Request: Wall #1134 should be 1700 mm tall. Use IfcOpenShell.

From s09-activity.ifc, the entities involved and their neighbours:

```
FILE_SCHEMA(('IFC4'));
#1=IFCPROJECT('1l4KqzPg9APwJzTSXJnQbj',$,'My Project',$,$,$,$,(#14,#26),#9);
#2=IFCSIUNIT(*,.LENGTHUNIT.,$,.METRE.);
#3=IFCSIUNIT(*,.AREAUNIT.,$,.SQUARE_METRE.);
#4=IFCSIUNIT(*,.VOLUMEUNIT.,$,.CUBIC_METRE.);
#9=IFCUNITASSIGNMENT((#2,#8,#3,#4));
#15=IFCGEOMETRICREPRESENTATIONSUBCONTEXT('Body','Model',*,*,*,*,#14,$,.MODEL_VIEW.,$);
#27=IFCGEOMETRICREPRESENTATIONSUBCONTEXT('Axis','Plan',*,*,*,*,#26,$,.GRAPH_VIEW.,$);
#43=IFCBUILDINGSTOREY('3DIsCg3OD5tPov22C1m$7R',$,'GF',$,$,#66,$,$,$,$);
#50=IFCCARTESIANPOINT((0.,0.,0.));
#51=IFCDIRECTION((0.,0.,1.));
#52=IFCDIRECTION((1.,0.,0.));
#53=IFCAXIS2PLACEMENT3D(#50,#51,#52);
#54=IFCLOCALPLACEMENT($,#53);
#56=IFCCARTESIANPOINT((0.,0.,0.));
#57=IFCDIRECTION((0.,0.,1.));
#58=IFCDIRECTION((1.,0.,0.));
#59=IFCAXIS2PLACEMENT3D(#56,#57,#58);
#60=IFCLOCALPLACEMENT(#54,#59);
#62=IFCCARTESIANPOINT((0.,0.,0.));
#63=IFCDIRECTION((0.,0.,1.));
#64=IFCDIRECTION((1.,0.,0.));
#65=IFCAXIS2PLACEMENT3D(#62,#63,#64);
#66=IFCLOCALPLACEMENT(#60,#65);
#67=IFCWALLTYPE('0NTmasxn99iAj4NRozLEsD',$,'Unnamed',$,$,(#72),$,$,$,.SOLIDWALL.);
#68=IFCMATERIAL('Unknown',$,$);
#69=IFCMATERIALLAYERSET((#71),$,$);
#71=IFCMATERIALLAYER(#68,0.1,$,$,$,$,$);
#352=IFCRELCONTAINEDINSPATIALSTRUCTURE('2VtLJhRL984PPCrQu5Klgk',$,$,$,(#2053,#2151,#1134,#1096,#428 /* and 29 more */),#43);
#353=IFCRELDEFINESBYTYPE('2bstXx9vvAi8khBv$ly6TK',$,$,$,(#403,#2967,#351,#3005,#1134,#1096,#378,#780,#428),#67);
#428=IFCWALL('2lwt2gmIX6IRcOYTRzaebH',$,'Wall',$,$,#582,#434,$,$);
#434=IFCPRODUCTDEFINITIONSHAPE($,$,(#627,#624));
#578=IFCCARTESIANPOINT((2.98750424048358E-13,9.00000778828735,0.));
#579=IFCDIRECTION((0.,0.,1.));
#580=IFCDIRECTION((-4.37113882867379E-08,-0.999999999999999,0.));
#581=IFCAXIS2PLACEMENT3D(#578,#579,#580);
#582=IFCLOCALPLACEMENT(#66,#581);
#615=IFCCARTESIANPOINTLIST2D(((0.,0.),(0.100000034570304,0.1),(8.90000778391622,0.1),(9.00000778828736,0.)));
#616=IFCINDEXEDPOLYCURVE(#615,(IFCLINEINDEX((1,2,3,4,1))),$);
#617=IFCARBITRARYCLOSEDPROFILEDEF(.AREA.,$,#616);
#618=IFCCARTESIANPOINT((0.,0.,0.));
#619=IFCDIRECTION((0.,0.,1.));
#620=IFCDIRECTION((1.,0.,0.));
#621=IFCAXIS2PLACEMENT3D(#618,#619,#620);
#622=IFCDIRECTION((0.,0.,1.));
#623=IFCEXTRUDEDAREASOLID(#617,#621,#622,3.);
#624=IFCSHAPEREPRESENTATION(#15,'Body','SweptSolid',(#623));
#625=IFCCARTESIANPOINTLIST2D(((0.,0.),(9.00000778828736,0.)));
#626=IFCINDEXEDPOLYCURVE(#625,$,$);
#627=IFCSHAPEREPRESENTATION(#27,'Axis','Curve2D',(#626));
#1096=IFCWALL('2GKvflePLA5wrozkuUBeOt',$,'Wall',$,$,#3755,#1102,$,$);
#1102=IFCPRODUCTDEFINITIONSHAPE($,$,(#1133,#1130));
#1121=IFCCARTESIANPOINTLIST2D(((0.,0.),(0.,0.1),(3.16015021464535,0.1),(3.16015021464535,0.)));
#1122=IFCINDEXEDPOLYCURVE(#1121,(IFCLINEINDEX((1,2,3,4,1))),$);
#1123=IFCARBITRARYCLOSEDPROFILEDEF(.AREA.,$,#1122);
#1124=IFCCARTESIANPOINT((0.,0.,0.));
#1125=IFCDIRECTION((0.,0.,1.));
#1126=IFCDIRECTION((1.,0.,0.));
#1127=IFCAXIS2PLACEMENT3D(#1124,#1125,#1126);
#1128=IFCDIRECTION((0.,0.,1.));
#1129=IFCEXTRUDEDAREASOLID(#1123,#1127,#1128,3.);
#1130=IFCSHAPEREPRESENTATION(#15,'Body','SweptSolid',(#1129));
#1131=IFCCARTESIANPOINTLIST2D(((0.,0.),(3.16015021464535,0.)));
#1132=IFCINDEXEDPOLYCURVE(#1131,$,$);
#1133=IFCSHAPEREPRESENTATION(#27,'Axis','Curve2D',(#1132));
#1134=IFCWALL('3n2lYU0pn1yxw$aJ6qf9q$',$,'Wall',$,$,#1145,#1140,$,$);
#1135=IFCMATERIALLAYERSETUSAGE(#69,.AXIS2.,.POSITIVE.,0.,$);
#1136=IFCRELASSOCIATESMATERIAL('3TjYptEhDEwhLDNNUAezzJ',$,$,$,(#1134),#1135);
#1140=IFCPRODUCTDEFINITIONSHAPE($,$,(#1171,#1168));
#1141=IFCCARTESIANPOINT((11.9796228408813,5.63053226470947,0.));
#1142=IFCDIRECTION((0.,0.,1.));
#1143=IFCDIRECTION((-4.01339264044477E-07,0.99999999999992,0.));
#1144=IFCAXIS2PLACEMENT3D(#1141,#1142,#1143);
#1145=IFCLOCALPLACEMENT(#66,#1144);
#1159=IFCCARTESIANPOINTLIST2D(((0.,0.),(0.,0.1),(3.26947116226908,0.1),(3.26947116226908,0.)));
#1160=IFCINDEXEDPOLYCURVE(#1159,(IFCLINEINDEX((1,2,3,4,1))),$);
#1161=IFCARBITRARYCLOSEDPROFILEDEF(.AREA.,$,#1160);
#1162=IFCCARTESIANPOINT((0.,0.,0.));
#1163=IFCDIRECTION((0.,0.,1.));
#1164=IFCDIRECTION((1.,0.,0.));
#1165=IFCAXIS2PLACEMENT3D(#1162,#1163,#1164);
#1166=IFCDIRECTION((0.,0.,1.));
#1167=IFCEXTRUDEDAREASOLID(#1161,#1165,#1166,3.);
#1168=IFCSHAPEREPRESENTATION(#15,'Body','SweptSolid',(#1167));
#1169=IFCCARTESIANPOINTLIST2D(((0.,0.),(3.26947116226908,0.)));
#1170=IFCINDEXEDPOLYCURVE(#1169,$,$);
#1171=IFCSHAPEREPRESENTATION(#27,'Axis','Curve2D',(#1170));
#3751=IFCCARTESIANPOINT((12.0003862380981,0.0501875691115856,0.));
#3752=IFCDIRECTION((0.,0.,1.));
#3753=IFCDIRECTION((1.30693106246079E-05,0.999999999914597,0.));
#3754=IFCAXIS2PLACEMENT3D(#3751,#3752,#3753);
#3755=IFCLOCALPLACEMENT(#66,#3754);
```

```python
import ifcopenshell
import ifcopenshell.geom
import ifcopenshell.util.representation
import ifcopenshell.util.shape
import ifcopenshell.util.unit

model = ifcopenshell.open("s09-activity.ifc")
unit_scale = ifcopenshell.util.unit.calculate_unit_scale(model)
settings = ifcopenshell.geom.settings()


def volume(element):
    """Net volume in cubic metres, openings subtracted."""
    shape = ifcopenshell.geom.create_shape(settings, element)
    return ifcopenshell.util.shape.get_volume(shape.geometry)


wall = model.by_guid("3n2lYU0pn1yxw$aJ6qf9q$")
before = volume(wall)

body = ifcopenshell.util.representation.get_representation(wall, "Model", "Body")
solid = body.Items[0]
old_height = solid.Depth
solid.Depth = 1.7 / unit_scale
after = volume(wall)

print(f"height {old_height:g} -> {solid.Depth:g}, volume {before:.3f} -> {after:.3f} m3")

model.write("s09-activity-out.ifc")
```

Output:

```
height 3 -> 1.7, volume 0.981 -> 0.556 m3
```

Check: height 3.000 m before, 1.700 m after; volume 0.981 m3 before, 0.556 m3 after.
